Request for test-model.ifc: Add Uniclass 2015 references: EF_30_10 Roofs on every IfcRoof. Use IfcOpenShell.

First a look at what the model holds.

```python
import ifcopenshell

model = ifcopenshell.open("test-model.ifc")
print(model.schema)
print("classifications:", [c.Name for c in model.by_type("IfcClassification")])
for ifc_class in ("IfcDoor", "IfcRoof", "IfcStair", "IfcWall", "IfcWindow"):
    print(ifc_class, len(model.by_type(ifc_class)))
```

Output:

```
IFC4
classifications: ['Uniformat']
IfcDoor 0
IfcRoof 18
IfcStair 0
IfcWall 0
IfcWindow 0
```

```python
import ifcopenshell
import ifcopenshell.api.classification

model = ifcopenshell.open("test-model.ifc")

system = ifcopenshell.api.classification.add_classification(model, classification="Uniclass 2015")

codes = {
    "IfcRoof": ("EF_30_10", "Roofs"),
}
for ifc_class, (code, name) in codes.items():
    products = model.by_type(ifc_class)
    ifcopenshell.api.classification.add_reference(
        model, products=products, classification=system, identification=code, name=name
    )
    print(code, len(products))

model.write("test-model_edited.ifc")
```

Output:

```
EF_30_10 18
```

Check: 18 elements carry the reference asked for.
